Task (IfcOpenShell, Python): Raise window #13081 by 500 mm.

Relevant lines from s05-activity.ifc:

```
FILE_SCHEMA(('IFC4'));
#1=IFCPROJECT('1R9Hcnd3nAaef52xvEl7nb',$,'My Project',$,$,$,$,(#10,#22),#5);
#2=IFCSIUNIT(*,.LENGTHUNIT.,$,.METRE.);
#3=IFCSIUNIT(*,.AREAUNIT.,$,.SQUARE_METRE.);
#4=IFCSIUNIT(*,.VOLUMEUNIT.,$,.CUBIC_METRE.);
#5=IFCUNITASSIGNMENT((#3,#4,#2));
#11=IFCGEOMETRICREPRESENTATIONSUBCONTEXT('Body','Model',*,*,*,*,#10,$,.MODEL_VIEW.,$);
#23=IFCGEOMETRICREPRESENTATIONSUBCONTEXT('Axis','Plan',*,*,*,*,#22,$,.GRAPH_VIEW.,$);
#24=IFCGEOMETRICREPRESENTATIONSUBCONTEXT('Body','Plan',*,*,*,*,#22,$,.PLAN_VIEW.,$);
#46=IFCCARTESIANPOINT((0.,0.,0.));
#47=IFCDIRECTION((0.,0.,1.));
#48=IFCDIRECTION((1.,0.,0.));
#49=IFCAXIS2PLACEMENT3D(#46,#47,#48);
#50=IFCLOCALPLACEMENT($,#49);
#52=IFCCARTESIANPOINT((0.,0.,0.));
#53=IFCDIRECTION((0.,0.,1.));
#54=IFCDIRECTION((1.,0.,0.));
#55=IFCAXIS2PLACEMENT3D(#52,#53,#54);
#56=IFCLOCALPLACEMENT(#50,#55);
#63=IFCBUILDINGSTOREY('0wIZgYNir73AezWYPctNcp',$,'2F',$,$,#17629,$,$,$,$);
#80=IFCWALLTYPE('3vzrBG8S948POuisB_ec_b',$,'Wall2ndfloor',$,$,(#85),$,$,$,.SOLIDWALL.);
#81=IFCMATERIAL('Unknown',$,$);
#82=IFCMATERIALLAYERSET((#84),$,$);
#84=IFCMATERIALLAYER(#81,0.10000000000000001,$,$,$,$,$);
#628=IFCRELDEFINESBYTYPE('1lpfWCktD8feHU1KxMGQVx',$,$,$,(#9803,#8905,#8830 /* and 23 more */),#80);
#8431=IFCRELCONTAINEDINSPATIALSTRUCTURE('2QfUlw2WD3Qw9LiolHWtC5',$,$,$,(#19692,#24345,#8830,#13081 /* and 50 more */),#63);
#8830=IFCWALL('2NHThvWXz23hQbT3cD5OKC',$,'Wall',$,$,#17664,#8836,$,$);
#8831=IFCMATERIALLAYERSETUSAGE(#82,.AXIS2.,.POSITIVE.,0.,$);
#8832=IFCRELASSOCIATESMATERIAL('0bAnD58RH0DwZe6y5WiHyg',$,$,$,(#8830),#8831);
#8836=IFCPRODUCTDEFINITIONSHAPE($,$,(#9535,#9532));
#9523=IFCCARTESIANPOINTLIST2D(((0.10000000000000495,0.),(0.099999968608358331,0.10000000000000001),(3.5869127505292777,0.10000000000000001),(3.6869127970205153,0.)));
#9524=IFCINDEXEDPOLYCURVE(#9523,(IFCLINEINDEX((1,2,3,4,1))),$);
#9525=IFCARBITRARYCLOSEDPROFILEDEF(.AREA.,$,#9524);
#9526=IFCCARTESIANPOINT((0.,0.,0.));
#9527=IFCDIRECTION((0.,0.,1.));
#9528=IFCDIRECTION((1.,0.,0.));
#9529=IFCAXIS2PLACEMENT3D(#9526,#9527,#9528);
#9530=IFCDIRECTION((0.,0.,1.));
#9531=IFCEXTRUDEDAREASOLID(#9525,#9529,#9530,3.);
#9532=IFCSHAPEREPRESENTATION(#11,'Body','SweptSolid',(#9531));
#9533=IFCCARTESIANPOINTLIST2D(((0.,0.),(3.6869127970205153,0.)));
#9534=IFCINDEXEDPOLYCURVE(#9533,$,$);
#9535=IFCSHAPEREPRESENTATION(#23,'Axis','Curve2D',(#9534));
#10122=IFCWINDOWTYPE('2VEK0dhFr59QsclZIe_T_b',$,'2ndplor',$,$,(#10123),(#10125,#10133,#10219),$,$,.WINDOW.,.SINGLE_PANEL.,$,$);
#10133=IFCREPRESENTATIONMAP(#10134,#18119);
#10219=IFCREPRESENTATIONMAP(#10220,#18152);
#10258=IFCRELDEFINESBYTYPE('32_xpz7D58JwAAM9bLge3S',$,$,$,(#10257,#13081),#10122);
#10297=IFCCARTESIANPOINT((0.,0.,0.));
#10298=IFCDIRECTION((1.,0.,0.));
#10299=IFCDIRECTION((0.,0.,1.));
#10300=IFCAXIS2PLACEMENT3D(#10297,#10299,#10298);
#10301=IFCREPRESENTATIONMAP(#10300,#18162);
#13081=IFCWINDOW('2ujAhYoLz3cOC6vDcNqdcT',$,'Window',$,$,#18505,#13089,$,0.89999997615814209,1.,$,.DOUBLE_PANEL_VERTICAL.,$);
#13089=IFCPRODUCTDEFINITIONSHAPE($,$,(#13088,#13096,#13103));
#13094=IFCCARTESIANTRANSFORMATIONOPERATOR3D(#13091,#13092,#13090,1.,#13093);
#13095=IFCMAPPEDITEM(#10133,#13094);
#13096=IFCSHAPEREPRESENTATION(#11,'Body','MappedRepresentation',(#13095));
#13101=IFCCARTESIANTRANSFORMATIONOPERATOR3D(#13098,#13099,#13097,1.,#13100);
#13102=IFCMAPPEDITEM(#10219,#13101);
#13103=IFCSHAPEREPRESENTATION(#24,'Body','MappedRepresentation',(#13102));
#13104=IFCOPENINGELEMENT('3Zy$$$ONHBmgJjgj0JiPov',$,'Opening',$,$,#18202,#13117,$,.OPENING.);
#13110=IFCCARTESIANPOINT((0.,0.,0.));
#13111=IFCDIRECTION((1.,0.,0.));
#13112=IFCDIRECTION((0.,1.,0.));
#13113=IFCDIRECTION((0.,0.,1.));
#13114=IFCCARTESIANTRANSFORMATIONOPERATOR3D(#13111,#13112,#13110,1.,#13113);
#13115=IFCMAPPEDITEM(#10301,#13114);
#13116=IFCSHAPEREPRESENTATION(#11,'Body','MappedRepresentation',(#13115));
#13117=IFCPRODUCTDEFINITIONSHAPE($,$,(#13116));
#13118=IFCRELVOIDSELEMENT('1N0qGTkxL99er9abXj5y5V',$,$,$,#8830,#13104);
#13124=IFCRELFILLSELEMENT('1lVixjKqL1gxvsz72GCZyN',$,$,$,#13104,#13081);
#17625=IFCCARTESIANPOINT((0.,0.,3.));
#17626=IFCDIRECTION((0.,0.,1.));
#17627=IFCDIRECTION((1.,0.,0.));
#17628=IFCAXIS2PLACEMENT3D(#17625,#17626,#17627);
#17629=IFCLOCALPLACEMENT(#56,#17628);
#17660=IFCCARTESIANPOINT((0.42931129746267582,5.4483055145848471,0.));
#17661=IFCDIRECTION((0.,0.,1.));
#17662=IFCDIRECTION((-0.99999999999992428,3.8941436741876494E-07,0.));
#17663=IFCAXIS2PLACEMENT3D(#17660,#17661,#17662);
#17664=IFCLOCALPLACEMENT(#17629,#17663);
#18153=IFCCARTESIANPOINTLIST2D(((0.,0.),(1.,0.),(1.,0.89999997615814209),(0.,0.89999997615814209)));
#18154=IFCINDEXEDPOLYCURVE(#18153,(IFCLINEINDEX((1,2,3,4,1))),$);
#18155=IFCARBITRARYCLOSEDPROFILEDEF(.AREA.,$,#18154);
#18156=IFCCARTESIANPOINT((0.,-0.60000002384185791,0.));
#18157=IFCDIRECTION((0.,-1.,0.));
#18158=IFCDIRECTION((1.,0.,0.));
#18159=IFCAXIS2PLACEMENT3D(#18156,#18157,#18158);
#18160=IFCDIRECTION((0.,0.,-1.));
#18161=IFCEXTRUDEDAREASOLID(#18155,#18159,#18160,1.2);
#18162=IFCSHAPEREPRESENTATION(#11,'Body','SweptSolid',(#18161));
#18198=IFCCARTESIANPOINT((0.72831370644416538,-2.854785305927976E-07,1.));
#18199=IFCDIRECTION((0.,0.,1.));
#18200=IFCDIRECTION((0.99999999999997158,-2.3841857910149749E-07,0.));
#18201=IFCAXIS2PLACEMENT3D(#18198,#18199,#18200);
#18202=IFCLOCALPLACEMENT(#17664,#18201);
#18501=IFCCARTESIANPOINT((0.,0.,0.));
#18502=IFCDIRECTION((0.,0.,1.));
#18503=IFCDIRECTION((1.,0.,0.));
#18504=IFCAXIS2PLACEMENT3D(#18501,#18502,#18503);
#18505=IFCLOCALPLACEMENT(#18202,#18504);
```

```python
import numpy as np
import ifcopenshell
import ifcopenshell.api.geometry
import ifcopenshell.util.placement
import ifcopenshell.util.unit

model = ifcopenshell.open("s05-activity.ifc")
unit_scale = ifcopenshell.util.unit.calculate_unit_scale(model)

window = model.by_guid("2ujAhYoLz3cOC6vDcNqdcT")
opening = window.FillsVoids[0].RelatingOpeningElement
dz = 0.5

shift = np.array([0.0, 0.0, dz])
# The window is placed relative to its opening, so it follows when the opening moves.
matrix = ifcopenshell.util.placement.get_local_placement(opening.ObjectPlacement)
matrix[:3, 3] += shift
ifcopenshell.api.geometry.edit_object_placement(
    model, product=opening, matrix=matrix, is_si=False, should_transform_children=True
)

print(f"moved by {dz * unit_scale:+.3f} m")

model.write("s05-activity_rev.ifc")
```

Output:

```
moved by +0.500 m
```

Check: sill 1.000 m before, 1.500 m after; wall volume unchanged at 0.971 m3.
